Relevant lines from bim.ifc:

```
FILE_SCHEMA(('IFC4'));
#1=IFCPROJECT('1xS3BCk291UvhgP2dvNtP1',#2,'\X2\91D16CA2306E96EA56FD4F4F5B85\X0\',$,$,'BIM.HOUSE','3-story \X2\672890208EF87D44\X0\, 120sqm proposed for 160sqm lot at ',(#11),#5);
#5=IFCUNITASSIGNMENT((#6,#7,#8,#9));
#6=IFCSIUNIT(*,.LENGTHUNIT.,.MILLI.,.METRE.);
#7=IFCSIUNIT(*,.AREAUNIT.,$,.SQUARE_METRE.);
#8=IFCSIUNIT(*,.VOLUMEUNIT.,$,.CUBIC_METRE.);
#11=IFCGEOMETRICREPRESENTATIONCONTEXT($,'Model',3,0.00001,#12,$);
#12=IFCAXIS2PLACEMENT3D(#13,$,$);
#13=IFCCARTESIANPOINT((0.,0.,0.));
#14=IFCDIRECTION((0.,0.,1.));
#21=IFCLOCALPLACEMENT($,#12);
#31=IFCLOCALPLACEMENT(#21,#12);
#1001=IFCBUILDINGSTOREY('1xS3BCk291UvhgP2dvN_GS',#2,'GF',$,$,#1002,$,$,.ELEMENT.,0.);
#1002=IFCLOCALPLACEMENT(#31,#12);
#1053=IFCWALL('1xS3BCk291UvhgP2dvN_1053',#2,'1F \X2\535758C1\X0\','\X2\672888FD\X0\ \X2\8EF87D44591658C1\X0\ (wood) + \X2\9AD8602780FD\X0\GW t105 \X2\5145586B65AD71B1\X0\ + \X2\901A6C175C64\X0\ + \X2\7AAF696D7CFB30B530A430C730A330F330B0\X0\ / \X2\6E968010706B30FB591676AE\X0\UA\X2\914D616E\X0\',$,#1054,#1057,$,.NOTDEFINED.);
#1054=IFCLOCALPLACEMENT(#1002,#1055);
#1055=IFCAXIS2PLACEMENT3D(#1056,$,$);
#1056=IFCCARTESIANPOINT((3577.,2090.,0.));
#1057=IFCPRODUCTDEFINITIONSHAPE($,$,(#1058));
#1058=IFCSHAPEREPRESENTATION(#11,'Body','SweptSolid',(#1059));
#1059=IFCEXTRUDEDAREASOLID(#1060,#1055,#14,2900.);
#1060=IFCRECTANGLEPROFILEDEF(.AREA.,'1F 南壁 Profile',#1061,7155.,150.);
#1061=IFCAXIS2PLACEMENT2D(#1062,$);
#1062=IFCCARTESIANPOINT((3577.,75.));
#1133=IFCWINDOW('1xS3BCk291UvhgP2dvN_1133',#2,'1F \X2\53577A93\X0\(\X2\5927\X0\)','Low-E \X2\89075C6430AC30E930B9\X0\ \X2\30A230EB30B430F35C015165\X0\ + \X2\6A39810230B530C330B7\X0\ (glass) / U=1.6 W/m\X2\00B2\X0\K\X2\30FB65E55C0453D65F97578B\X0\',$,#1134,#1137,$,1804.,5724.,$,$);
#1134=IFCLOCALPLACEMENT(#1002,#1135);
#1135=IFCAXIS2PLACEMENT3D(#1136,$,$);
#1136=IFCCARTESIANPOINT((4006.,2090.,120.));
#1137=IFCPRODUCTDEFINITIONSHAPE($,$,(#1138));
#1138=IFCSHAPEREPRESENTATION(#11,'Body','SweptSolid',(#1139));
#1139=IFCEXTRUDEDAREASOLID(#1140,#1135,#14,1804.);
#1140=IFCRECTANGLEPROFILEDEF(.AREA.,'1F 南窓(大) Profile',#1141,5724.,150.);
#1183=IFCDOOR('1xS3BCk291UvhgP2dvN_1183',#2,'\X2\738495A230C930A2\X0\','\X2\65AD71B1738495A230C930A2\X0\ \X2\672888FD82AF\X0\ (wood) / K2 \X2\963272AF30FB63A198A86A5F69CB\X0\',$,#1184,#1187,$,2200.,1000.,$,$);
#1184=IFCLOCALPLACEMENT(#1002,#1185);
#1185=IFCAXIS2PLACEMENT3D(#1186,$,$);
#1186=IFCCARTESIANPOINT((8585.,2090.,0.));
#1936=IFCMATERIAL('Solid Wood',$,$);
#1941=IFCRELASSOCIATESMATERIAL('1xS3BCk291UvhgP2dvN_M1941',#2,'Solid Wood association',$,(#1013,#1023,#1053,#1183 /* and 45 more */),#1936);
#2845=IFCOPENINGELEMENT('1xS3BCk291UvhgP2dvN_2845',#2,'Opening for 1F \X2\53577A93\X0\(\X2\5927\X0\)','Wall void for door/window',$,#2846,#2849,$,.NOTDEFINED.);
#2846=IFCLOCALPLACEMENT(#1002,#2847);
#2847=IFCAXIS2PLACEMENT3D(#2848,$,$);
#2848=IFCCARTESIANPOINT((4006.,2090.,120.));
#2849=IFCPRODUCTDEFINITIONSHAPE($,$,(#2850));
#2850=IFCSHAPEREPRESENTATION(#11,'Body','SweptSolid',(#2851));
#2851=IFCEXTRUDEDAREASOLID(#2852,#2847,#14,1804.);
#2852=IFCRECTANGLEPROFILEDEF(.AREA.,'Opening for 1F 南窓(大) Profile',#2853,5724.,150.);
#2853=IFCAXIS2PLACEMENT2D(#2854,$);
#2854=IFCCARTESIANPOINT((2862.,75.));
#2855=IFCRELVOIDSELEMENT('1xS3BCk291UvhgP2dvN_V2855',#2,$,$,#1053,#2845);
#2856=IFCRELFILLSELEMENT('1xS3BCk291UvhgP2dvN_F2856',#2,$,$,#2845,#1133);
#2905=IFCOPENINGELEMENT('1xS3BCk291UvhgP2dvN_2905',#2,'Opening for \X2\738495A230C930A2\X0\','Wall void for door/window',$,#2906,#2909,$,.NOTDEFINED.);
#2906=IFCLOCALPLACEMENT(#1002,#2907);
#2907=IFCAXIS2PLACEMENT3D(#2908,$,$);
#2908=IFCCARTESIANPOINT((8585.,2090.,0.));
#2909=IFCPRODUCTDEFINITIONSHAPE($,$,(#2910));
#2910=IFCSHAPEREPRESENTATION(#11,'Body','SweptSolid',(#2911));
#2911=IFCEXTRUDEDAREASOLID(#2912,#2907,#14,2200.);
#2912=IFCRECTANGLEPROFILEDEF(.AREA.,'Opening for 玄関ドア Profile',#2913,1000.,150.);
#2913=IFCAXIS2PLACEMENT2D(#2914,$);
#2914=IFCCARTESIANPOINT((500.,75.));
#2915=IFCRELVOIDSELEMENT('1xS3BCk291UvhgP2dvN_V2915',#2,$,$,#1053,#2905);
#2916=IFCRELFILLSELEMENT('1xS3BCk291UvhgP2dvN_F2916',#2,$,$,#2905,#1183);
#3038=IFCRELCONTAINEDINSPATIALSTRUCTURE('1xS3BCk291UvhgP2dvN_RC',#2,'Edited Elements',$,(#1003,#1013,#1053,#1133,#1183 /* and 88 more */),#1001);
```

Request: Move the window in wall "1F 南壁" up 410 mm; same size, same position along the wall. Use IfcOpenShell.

```python
import numpy as np
import ifcopenshell
import ifcopenshell.api.geometry
import ifcopenshell.util.placement
import ifcopenshell.util.unit

model = ifcopenshell.open("bim.ifc")
unit_scale = ifcopenshell.util.unit.calculate_unit_scale(model)

window = model.by_guid("1xS3BCk291UvhgP2dvN_1133")
opening = window.FillsVoids[0].RelatingOpeningElement
dz = 410.0

shift = np.array([0.0, 0.0, dz])
# The window is not placed relative to its opening, so move both.
for product in (opening, window):
    matrix = ifcopenshell.util.placement.get_local_placement(product.ObjectPlacement)
    matrix[:3, 3] += shift
    ifcopenshell.api.geometry.edit_object_placement(model, product=product, matrix=matrix, is_si=False)

print(f"moved by {dz * unit_scale:+.3f} m")

model.write("bim_edited.ifc")
```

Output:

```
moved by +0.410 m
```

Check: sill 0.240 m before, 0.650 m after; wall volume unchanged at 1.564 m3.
